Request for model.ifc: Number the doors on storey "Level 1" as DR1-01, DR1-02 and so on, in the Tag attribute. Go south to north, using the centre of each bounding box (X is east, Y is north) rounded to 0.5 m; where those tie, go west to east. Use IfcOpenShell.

First a look at what the model holds.

```python
import ifcopenshell
import ifcopenshell.util.element
import ifcopenshell.util.placement

model = ifcopenshell.open("model.ifc")
print(model.schema)
storey = next(s for s in model.by_type("IfcBuildingStorey") if s.Name == "Level 1")
doors = [e for e in ifcopenshell.util.element.get_decomposition(storey) if e.is_a("IfcDoor")]
for e in sorted(doors, key=lambda e: e.id()):
    origin = ifcopenshell.util.placement.get_local_placement(e.ObjectPlacement)[:3, 3]
    print(e.id(), e.Tag, e.Name, origin.round(2) + 0.0, sep=" | ")
```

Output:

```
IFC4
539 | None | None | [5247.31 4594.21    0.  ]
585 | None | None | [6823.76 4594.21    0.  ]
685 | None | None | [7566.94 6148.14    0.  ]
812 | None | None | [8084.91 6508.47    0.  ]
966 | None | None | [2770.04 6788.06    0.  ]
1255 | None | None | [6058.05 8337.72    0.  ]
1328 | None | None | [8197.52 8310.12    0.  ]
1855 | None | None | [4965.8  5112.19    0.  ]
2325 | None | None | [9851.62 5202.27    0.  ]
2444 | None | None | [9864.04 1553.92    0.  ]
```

```python
import ifcopenshell
import ifcopenshell.geom
import ifcopenshell.util.element
import ifcopenshell.util.shape

model = ifcopenshell.open("model.ifc")
settings = ifcopenshell.geom.settings()
settings.set("use-world-coords", True)


def centre(element):
    shape = ifcopenshell.geom.create_shape(settings, element)
    return ifcopenshell.util.shape.get_bbox_centroid(shape.geometry)


storey = next(s for s in model.by_type("IfcBuildingStorey") if s.Name == "Level 1")
doors = [e for e in ifcopenshell.util.element.get_decomposition(storey) if e.is_a("IfcDoor")]

# Insertion points can sit at a corner or the storey origin, so sort by the geometry (in metres).
centres = {e: centre(e) for e in doors}
doors.sort(key=lambda e: (round(centres[e][1] / 0.5), centres[e][0]))

for i, e in enumerate(doors, start=1):
    number = f"DR1-{i:02d}"
    e.Tag = number
    print(e.id(), number)

model.write("model_v2.ifc")
```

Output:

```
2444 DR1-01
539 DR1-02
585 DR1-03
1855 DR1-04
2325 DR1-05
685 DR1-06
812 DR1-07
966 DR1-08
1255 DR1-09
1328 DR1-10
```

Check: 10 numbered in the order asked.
